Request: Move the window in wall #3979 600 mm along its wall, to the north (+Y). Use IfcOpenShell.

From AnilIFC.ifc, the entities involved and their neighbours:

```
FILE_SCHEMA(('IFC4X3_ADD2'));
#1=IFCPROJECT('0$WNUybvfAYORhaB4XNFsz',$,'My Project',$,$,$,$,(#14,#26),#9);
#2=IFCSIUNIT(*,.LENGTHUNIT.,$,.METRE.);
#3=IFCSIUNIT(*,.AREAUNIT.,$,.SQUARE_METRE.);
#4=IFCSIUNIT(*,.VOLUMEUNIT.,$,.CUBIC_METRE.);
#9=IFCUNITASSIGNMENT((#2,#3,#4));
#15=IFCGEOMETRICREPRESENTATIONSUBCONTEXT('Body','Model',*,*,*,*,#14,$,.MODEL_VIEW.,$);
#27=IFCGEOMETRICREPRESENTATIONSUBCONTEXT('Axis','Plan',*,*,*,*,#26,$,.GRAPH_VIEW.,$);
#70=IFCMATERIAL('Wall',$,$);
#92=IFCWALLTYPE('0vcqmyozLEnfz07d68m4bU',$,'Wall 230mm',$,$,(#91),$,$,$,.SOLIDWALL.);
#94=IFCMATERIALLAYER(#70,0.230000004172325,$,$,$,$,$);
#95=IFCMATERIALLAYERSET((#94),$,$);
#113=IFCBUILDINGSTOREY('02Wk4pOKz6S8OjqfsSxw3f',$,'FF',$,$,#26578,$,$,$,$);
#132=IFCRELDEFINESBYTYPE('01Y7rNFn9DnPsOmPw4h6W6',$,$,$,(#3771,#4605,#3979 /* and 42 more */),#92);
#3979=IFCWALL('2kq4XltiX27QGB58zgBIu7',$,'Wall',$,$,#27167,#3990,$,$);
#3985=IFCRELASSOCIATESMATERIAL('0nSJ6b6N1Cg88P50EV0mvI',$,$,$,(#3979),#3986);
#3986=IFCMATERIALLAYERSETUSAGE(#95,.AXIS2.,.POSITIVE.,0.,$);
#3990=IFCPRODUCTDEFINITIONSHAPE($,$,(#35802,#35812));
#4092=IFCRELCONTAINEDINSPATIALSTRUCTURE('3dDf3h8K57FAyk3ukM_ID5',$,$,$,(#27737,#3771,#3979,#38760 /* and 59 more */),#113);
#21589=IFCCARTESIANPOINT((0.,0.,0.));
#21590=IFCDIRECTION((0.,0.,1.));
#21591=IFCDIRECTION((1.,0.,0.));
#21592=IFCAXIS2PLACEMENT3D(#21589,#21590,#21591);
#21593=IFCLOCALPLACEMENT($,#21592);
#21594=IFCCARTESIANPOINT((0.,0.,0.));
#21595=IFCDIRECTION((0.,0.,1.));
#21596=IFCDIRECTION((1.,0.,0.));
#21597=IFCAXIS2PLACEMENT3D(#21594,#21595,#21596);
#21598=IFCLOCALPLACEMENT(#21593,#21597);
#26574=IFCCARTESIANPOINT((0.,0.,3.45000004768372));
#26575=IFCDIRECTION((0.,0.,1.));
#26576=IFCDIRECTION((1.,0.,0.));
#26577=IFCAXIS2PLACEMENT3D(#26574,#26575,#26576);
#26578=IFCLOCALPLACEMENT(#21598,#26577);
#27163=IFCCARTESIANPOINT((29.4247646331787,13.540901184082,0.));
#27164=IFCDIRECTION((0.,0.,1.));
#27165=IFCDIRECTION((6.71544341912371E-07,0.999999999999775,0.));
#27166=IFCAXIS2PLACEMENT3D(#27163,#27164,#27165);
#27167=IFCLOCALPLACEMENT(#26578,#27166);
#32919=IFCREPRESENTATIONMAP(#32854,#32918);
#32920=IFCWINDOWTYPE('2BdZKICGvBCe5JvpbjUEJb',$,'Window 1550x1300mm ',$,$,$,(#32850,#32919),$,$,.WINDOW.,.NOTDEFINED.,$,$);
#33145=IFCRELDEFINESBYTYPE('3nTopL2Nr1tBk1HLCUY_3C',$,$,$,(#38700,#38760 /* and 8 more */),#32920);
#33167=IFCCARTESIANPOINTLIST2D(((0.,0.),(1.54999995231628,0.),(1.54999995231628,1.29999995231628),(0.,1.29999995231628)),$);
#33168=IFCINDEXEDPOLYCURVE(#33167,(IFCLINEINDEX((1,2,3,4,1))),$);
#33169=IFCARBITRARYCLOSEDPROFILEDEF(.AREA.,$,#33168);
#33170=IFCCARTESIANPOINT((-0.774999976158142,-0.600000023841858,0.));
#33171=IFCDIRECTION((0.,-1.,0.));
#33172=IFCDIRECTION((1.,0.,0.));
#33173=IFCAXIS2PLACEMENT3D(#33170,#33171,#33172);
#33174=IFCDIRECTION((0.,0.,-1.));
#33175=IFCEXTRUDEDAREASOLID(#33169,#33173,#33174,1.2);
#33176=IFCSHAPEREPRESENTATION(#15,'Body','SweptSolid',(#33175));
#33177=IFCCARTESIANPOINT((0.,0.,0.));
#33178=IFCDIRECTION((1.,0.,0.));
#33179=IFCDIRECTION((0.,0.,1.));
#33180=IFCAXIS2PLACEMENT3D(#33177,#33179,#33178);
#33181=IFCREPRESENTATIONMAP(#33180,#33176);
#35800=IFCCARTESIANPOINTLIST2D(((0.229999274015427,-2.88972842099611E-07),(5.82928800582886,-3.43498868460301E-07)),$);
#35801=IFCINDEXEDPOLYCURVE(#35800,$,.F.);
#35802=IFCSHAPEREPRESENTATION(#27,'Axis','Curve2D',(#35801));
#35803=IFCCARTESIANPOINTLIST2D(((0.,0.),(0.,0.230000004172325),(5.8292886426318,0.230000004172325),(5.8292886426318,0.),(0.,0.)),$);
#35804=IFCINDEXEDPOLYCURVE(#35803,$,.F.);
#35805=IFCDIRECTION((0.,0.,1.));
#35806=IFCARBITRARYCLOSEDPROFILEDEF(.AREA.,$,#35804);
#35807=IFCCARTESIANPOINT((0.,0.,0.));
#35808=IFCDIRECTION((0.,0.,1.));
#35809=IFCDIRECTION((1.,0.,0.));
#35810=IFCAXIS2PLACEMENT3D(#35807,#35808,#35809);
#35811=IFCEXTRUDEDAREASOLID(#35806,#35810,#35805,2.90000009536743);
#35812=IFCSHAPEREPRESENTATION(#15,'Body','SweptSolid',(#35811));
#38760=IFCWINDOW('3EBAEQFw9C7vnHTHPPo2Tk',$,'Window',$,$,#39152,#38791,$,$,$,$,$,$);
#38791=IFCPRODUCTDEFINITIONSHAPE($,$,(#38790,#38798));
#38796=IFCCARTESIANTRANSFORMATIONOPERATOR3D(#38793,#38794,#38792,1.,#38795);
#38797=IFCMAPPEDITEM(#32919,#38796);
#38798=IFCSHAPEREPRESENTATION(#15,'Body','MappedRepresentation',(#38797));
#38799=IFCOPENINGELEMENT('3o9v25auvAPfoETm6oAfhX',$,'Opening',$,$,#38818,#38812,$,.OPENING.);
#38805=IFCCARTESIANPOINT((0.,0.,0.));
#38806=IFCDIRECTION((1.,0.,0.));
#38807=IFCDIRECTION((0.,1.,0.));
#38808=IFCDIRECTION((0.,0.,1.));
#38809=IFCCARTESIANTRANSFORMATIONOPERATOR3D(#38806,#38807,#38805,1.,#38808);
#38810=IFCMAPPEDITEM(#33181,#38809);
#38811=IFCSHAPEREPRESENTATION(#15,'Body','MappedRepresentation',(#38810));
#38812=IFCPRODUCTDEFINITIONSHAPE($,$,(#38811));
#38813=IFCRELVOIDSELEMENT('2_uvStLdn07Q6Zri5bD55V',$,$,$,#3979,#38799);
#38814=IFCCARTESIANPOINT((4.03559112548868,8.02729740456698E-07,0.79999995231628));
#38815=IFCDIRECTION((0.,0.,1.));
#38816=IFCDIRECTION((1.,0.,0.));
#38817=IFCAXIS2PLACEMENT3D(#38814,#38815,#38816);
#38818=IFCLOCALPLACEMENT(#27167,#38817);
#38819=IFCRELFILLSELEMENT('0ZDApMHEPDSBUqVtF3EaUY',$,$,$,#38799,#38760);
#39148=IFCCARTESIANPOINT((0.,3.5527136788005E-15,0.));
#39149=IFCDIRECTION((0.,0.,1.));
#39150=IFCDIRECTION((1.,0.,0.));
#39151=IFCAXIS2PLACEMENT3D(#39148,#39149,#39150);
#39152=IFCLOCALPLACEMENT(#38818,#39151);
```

```python
import ifcopenshell
import ifcopenshell.api.geometry
import ifcopenshell.util.placement
import ifcopenshell.util.unit

model = ifcopenshell.open("AnilIFC.ifc")
unit_scale = ifcopenshell.util.unit.calculate_unit_scale(model)

window = model.by_guid("3EBAEQFw9C7vnHTHPPo2Tk")
opening = window.FillsVoids[0].RelatingOpeningElement
wall = opening.VoidsElements[0].RelatingBuildingElement

wall_matrix = ifcopenshell.util.placement.get_local_placement(wall.ObjectPlacement)
shift = wall_matrix[:3, 0] * 0.6 / unit_scale
before = ifcopenshell.util.placement.get_local_placement(window.ObjectPlacement)[:3, 3].copy()

# The window is placed relative to its opening, so it follows when the opening moves.
matrix = ifcopenshell.util.placement.get_local_placement(opening.ObjectPlacement)
matrix[:3, 3] += shift
ifcopenshell.api.geometry.edit_object_placement(
    model, product=opening, matrix=matrix, is_si=False, should_transform_children=True
)

after = ifcopenshell.util.placement.get_local_placement(window.ObjectPlacement)[:3, 3]
print("window moved by", (after - before).round(3) + 0.0)

model.write("AnilIFC_edited.ifc")
```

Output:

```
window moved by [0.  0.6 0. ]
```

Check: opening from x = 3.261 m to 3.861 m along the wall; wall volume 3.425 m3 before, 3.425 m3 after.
